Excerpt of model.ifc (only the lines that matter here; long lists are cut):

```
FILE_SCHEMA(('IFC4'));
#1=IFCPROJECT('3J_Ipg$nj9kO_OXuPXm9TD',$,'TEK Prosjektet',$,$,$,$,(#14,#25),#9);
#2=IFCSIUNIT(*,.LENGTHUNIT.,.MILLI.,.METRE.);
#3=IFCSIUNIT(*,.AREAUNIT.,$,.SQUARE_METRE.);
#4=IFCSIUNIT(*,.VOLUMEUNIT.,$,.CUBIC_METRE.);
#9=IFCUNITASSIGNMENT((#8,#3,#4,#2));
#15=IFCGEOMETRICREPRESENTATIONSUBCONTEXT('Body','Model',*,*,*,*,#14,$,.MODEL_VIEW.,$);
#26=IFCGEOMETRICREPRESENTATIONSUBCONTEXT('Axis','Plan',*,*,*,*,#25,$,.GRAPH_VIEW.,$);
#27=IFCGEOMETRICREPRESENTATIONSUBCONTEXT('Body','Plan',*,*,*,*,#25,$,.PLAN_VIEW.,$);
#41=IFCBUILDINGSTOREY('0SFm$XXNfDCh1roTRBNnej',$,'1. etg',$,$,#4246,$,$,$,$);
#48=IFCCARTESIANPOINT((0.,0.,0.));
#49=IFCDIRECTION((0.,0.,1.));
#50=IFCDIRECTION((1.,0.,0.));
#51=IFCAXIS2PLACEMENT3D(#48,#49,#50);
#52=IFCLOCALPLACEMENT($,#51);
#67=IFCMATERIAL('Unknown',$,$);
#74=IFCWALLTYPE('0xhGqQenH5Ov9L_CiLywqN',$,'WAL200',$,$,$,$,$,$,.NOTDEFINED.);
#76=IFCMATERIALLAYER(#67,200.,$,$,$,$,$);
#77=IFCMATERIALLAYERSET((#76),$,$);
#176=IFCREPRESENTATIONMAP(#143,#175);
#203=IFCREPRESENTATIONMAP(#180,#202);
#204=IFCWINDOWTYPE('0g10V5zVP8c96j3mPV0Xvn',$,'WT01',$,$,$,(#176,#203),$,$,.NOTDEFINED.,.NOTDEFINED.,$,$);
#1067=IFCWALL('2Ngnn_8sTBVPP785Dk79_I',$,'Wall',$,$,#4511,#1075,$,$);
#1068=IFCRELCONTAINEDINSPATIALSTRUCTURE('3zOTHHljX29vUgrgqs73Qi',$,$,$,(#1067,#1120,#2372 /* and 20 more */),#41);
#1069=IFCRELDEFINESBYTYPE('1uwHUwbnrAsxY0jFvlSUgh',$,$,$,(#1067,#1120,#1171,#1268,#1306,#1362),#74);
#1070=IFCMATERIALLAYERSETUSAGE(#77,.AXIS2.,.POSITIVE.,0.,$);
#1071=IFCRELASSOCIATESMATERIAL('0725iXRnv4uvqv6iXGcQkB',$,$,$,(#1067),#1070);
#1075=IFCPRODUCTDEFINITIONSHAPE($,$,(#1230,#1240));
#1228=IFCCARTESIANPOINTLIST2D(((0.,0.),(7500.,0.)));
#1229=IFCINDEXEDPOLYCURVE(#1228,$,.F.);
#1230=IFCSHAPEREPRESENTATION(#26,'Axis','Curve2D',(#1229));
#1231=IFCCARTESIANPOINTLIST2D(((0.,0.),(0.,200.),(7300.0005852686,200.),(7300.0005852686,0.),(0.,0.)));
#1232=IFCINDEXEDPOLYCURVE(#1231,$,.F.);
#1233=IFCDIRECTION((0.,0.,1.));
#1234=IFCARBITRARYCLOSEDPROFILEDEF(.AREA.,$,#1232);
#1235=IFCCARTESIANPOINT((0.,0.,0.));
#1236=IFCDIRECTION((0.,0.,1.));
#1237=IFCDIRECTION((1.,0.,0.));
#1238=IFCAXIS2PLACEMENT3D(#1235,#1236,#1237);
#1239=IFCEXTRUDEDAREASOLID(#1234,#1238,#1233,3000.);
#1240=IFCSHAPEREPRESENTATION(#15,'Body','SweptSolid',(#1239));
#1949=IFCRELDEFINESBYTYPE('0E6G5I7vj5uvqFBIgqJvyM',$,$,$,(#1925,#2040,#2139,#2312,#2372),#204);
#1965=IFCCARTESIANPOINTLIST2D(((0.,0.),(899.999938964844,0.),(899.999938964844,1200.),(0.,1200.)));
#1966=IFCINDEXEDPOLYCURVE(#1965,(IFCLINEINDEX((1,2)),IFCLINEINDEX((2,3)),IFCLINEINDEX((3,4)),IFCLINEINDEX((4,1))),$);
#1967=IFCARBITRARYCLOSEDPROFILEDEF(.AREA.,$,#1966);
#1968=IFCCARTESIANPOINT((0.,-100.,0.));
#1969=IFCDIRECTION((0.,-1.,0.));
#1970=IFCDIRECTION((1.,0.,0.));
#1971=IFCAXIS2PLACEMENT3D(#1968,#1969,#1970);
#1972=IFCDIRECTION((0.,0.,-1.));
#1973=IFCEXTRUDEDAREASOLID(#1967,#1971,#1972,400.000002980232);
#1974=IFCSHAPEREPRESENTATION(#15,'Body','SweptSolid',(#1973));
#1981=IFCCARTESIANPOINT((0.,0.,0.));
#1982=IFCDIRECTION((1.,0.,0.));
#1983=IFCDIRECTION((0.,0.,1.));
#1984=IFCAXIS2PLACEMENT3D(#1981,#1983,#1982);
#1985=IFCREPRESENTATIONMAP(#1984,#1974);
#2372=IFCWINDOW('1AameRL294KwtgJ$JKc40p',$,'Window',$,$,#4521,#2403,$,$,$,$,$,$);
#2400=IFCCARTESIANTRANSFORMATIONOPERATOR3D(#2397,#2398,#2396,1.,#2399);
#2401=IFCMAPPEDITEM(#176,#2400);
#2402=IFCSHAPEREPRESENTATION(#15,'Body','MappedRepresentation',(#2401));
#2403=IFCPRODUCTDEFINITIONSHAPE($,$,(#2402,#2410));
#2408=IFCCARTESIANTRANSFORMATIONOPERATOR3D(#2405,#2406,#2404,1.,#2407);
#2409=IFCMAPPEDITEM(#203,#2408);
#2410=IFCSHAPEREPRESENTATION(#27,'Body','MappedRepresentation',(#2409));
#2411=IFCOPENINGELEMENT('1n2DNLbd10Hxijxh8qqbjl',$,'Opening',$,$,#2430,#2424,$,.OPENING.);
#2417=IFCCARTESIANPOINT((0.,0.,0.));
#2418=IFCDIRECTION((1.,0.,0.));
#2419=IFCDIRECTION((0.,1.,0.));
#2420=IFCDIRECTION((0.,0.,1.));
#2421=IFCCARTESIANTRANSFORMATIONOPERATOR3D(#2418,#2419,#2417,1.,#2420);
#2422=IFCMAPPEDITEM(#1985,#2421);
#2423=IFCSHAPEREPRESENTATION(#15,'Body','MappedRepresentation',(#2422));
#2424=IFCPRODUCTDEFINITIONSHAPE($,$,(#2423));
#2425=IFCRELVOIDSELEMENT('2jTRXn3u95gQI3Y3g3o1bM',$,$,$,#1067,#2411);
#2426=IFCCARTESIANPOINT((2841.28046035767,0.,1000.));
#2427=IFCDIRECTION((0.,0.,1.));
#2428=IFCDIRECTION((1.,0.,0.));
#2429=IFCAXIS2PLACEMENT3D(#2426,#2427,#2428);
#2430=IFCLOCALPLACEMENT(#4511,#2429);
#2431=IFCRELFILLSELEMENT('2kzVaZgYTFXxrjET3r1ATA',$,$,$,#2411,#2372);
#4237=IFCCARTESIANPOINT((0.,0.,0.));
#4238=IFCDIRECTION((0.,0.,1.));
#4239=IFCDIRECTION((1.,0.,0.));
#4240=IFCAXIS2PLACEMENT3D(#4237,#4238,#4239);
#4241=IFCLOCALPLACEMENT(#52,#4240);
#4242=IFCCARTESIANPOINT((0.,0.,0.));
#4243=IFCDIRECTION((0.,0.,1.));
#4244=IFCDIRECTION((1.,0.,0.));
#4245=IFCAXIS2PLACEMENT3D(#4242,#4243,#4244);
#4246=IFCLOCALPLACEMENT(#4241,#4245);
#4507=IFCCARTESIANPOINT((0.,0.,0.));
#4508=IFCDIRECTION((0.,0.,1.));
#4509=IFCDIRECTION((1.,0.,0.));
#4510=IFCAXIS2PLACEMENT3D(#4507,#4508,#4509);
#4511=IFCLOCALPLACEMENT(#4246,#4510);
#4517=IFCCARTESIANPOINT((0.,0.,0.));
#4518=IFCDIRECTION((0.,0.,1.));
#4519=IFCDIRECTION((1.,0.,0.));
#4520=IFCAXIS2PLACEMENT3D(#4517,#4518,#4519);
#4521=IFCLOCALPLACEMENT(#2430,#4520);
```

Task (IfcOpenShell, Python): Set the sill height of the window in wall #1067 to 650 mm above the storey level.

```python
import numpy as np
import ifcopenshell
import ifcopenshell.api.geometry
import ifcopenshell.geom
import ifcopenshell.util.element
import ifcopenshell.util.placement
import ifcopenshell.util.shape
import ifcopenshell.util.unit

model = ifcopenshell.open("model.ifc")
unit_scale = ifcopenshell.util.unit.calculate_unit_scale(model)

window = model.by_guid("1AameRL294KwtgJ$JKc40p")
opening = window.FillsVoids[0].RelatingOpeningElement
storey = ifcopenshell.util.element.get_container(window, ifc_class="IfcBuildingStorey")
level = ifcopenshell.util.placement.get_local_placement(storey.ObjectPlacement)[2, 3]

# The opening's origin need not be at the sill, so measure its lowest point.
shape = ifcopenshell.geom.create_shape(ifcopenshell.geom.settings(), opening)
bottom = ifcopenshell.util.shape.get_shape_bottom_elevation(shape, shape.geometry) / unit_scale
dz = level + 650.0 - bottom

shift = np.array([0.0, 0.0, dz])
# The window is placed relative to its opening, so it follows when the opening moves.
matrix = ifcopenshell.util.placement.get_local_placement(opening.ObjectPlacement)
matrix[:3, 3] += shift
ifcopenshell.api.geometry.edit_object_placement(
    model, product=opening, matrix=matrix, is_si=False, should_transform_children=True
)

print(f"moved by {dz * unit_scale:+.3f} m")

model.write("model_v2.ifc")
```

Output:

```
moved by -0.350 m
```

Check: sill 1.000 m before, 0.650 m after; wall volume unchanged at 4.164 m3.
